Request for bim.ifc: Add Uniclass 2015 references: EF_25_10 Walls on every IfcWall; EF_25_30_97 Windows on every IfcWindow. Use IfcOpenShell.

First a look at what the model holds.

```python
import ifcopenshell

model = ifcopenshell.open("bim.ifc")
print(model.schema)
print("classifications:", [c.Name for c in model.by_type("IfcClassification")])
for ifc_class in ("IfcDoor", "IfcRoof", "IfcStair", "IfcWall", "IfcWindow"):
    print(ifc_class, len(model.by_type(ifc_class)))
```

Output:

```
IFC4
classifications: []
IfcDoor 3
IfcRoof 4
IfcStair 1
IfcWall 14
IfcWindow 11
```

```python
import ifcopenshell
import ifcopenshell.api.classification

model = ifcopenshell.open("bim.ifc")

system = ifcopenshell.api.classification.add_classification(model, classification="Uniclass 2015")

codes = {
    "IfcWall": ("EF_25_10", "Walls"),
    "IfcWindow": ("EF_25_30_97", "Windows"),
}
for ifc_class, (code, name) in codes.items():
    products = model.by_type(ifc_class)
    ifcopenshell.api.classification.add_reference(
        model, products=products, classification=system, identification=code, name=name
    )
    print(code, len(products))

model.write("bim_edited.ifc")
```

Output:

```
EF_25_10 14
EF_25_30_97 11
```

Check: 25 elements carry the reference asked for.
